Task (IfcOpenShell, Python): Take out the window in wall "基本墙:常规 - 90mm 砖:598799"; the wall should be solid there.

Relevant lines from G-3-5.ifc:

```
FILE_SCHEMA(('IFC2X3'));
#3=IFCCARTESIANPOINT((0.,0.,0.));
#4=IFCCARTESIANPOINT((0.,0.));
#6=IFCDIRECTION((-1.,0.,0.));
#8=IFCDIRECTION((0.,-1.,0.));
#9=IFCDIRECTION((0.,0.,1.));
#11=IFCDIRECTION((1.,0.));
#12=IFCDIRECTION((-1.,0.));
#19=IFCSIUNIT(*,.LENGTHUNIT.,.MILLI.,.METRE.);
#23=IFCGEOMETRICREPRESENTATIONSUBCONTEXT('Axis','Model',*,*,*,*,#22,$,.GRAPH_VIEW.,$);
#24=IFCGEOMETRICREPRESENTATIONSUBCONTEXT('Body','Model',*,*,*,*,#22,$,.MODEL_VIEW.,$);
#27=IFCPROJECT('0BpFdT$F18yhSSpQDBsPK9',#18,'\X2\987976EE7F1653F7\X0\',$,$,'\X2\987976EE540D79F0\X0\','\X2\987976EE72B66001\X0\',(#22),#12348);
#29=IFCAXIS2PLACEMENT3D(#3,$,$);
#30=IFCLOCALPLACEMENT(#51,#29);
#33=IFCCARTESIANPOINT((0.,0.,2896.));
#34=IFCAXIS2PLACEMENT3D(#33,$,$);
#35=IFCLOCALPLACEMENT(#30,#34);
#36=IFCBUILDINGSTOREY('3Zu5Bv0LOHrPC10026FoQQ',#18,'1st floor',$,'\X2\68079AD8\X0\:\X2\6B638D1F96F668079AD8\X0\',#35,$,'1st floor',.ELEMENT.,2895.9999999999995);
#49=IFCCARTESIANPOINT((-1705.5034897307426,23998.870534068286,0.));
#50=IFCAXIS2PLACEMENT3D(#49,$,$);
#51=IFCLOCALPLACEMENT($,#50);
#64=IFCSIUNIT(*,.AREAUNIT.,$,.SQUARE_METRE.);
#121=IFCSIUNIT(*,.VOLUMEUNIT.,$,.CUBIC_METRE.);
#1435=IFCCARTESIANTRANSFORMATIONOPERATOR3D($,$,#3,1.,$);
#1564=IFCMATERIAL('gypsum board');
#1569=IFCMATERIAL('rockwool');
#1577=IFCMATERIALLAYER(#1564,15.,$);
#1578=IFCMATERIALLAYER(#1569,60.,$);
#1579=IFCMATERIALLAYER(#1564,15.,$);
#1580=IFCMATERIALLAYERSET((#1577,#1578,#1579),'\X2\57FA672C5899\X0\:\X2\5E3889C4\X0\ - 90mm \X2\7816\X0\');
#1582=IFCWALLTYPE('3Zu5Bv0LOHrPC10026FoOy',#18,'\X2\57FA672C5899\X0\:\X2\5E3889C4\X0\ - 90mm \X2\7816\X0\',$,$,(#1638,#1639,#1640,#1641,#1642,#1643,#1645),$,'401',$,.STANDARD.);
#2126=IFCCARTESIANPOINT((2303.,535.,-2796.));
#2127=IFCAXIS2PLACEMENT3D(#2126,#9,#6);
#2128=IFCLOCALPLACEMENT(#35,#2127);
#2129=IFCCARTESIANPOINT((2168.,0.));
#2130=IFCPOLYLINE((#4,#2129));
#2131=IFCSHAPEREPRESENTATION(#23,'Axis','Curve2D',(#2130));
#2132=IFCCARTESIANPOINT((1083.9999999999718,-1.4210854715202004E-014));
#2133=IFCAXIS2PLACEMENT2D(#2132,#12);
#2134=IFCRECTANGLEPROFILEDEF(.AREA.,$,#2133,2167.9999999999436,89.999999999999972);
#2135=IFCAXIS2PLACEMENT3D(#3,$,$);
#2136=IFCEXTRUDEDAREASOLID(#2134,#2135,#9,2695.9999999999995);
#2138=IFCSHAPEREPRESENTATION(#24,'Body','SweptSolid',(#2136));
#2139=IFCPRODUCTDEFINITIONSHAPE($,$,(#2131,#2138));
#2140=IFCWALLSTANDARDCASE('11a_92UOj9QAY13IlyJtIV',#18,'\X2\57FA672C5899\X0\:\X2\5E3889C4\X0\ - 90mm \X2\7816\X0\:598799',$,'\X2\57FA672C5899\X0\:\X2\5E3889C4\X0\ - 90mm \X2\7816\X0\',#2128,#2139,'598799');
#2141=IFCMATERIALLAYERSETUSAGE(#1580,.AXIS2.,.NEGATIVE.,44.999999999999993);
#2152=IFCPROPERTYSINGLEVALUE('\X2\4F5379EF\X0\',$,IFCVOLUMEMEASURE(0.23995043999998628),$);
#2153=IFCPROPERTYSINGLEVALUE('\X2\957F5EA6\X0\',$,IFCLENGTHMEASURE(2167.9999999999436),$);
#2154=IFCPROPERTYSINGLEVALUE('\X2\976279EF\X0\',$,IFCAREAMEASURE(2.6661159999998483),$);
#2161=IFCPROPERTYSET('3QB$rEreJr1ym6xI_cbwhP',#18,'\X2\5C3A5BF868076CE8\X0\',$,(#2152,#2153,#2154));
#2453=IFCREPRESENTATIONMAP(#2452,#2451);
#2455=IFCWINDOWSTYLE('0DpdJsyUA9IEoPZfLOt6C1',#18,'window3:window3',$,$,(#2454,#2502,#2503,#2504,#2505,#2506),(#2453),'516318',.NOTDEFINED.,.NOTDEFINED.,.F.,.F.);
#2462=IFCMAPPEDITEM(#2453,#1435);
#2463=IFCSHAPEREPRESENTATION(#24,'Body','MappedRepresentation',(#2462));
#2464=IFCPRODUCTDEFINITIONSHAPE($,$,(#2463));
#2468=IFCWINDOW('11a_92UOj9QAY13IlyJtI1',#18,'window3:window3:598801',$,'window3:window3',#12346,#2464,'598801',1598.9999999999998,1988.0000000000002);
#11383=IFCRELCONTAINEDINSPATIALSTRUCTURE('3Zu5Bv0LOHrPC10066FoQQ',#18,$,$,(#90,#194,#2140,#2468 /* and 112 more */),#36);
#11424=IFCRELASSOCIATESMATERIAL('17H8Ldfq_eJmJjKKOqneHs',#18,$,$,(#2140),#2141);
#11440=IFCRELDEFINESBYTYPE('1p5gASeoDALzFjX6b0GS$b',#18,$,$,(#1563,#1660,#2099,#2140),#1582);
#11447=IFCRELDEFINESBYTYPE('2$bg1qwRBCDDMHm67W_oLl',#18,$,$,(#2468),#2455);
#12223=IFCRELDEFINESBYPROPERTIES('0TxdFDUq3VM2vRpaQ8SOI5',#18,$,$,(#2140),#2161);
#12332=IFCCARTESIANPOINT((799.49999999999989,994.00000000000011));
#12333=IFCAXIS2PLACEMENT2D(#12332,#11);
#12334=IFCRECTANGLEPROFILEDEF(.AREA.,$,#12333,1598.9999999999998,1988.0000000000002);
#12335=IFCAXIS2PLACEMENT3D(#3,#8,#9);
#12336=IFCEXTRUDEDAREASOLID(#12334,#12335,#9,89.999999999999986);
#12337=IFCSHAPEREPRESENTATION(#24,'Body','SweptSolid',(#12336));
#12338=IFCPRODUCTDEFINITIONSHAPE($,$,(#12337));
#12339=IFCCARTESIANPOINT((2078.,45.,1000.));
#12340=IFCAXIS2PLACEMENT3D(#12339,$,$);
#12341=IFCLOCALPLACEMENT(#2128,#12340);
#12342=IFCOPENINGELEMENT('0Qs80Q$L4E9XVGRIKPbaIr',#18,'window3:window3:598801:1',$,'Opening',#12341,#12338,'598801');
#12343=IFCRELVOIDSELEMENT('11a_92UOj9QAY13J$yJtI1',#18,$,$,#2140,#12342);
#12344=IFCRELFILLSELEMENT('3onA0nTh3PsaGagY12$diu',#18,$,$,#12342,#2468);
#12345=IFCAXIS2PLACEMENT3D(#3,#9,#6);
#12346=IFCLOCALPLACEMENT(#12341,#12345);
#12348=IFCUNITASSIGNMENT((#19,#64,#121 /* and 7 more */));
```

```python
import ifcopenshell
import ifcopenshell.api.feature
import ifcopenshell.api.pset
import ifcopenshell.api.root
import ifcopenshell.geom
import ifcopenshell.util.element
import ifcopenshell.util.shape
import ifcopenshell.util.unit

model = ifcopenshell.open("G-3-5.ifc")
area_scale = ifcopenshell.util.unit.calculate_unit_scale(model, "AREAUNIT")
volume_scale = ifcopenshell.util.unit.calculate_unit_scale(model, "VOLUMEUNIT")
settings = ifcopenshell.geom.settings()


def volume(element):
    """Net volume in cubic metres, openings subtracted."""
    shape = ifcopenshell.geom.create_shape(settings, element)
    return ifcopenshell.util.shape.get_volume(shape.geometry)


window = model.by_guid("11a_92UOj9QAY13IlyJtI1")
opening = window.FillsVoids[0].RelatingOpeningElement
wall = opening.VoidsElements[0].RelatingBuildingElement
before = volume(wall)

ifcopenshell.api.root.remove_product(model, product=window)
ifcopenshell.api.feature.remove_feature(model, feature=opening)

after = volume(wall)
thickness = 0.09  # wall thickness in metres

# Update the wall's stored quantities.
pset = model.by_id(ifcopenshell.util.element.get_pset(wall, "尺寸标注", should_inherit=False)["id"])
ifcopenshell.api.pset.edit_pset(model, pset=pset, properties={
    "体积": model.create_entity("IfcVolumeMeasure", after / volume_scale),
    "面积": model.create_entity("IfcAreaMeasure", after / thickness / area_scale),
})

print(f"wall volume {before:.3f} -> {after:.3f} m3")

model.write("G-3-5_edited.ifc")
```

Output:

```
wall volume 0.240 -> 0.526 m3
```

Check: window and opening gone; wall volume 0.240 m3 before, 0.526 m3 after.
